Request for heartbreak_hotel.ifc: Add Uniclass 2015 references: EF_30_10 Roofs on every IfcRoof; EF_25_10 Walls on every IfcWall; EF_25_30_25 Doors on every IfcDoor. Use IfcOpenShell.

First a look at what the model holds.

```python
import ifcopenshell

model = ifcopenshell.open("heartbreak_hotel.ifc")
print(model.schema)
print("classifications:", [c.Name for c in model.by_type("IfcClassification")])
for ifc_class in ("IfcDoor", "IfcRoof", "IfcStair", "IfcWall", "IfcWindow"):
    print(ifc_class, len(model.by_type(ifc_class)))
```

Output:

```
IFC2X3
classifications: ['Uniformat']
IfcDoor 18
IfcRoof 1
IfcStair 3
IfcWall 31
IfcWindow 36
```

```python
import ifcopenshell
import ifcopenshell.api.classification

model = ifcopenshell.open("heartbreak_hotel.ifc")

# IFC2X3 requires Source and Edition and has no link from the project to the system.
system = model.create_entity("IfcClassification", Source="NBS", Edition="2015", Name="Uniclass 2015")

codes = {
    "IfcRoof": ("EF_30_10", "Roofs"),
    "IfcWall": ("EF_25_10", "Walls"),
    "IfcDoor": ("EF_25_30_25", "Doors"),
}
for ifc_class, (code, name) in codes.items():
    products = model.by_type(ifc_class)
    ifcopenshell.api.classification.add_reference(
        model, products=products, classification=system, identification=code, name=name
    )
    print(code, len(products))

model.write("heartbreak_hotel_rev.ifc")
```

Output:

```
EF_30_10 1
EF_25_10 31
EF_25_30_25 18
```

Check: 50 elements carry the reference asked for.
